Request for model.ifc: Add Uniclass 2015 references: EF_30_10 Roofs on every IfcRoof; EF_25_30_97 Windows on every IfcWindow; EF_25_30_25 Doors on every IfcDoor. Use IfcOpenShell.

First a look at what the model holds.

```python
import ifcopenshell

model = ifcopenshell.open("model.ifc")
print(model.schema)
print("classifications:", [c.Name for c in model.by_type("IfcClassification")])
for ifc_class in ("IfcDoor", "IfcRoof", "IfcStair", "IfcWall", "IfcWindow"):
    print(ifc_class, len(model.by_type(ifc_class)))
```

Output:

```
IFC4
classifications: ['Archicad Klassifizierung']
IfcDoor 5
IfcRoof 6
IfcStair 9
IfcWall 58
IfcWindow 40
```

```python
import ifcopenshell
import ifcopenshell.api.classification

model = ifcopenshell.open("model.ifc")

system = ifcopenshell.api.classification.add_classification(model, classification="Uniclass 2015")

codes = {
    "IfcRoof": ("EF_30_10", "Roofs"),
    "IfcWindow": ("EF_25_30_97", "Windows"),
    "IfcDoor": ("EF_25_30_25", "Doors"),
}
for ifc_class, (code, name) in codes.items():
    products = model.by_type(ifc_class)
    ifcopenshell.api.classification.add_reference(
        model, products=products, classification=system, identification=code, name=name
    )
    print(code, len(products))

model.write("model_edited.ifc")
```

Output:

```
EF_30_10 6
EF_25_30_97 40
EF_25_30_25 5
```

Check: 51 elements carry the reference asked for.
